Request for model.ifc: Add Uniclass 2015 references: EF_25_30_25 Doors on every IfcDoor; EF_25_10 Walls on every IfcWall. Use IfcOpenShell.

First a look at what the model holds.

```python
import ifcopenshell

model = ifcopenshell.open("model.ifc")
print(model.schema)
print("classifications:", [c.Name for c in model.by_type("IfcClassification")])
for ifc_class in ("IfcDoor", "IfcRoof", "IfcStair", "IfcWall", "IfcWindow"):
    print(ifc_class, len(model.by_type(ifc_class)))
```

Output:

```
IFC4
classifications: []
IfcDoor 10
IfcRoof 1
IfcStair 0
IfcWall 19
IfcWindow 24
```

```python
import ifcopenshell
import ifcopenshell.api.classification

model = ifcopenshell.open("model.ifc")

system = ifcopenshell.api.classification.add_classification(model, classification="Uniclass 2015")

codes = {
    "IfcDoor": ("EF_25_30_25", "Doors"),
    "IfcWall": ("EF_25_10", "Walls"),
}
for ifc_class, (code, name) in codes.items():
    products = model.by_type(ifc_class)
    ifcopenshell.api.classification.add_reference(
        model, products=products, classification=system, identification=code, name=name
    )
    print(code, len(products))

model.write("model_edited.ifc")
```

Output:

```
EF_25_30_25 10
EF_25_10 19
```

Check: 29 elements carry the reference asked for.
